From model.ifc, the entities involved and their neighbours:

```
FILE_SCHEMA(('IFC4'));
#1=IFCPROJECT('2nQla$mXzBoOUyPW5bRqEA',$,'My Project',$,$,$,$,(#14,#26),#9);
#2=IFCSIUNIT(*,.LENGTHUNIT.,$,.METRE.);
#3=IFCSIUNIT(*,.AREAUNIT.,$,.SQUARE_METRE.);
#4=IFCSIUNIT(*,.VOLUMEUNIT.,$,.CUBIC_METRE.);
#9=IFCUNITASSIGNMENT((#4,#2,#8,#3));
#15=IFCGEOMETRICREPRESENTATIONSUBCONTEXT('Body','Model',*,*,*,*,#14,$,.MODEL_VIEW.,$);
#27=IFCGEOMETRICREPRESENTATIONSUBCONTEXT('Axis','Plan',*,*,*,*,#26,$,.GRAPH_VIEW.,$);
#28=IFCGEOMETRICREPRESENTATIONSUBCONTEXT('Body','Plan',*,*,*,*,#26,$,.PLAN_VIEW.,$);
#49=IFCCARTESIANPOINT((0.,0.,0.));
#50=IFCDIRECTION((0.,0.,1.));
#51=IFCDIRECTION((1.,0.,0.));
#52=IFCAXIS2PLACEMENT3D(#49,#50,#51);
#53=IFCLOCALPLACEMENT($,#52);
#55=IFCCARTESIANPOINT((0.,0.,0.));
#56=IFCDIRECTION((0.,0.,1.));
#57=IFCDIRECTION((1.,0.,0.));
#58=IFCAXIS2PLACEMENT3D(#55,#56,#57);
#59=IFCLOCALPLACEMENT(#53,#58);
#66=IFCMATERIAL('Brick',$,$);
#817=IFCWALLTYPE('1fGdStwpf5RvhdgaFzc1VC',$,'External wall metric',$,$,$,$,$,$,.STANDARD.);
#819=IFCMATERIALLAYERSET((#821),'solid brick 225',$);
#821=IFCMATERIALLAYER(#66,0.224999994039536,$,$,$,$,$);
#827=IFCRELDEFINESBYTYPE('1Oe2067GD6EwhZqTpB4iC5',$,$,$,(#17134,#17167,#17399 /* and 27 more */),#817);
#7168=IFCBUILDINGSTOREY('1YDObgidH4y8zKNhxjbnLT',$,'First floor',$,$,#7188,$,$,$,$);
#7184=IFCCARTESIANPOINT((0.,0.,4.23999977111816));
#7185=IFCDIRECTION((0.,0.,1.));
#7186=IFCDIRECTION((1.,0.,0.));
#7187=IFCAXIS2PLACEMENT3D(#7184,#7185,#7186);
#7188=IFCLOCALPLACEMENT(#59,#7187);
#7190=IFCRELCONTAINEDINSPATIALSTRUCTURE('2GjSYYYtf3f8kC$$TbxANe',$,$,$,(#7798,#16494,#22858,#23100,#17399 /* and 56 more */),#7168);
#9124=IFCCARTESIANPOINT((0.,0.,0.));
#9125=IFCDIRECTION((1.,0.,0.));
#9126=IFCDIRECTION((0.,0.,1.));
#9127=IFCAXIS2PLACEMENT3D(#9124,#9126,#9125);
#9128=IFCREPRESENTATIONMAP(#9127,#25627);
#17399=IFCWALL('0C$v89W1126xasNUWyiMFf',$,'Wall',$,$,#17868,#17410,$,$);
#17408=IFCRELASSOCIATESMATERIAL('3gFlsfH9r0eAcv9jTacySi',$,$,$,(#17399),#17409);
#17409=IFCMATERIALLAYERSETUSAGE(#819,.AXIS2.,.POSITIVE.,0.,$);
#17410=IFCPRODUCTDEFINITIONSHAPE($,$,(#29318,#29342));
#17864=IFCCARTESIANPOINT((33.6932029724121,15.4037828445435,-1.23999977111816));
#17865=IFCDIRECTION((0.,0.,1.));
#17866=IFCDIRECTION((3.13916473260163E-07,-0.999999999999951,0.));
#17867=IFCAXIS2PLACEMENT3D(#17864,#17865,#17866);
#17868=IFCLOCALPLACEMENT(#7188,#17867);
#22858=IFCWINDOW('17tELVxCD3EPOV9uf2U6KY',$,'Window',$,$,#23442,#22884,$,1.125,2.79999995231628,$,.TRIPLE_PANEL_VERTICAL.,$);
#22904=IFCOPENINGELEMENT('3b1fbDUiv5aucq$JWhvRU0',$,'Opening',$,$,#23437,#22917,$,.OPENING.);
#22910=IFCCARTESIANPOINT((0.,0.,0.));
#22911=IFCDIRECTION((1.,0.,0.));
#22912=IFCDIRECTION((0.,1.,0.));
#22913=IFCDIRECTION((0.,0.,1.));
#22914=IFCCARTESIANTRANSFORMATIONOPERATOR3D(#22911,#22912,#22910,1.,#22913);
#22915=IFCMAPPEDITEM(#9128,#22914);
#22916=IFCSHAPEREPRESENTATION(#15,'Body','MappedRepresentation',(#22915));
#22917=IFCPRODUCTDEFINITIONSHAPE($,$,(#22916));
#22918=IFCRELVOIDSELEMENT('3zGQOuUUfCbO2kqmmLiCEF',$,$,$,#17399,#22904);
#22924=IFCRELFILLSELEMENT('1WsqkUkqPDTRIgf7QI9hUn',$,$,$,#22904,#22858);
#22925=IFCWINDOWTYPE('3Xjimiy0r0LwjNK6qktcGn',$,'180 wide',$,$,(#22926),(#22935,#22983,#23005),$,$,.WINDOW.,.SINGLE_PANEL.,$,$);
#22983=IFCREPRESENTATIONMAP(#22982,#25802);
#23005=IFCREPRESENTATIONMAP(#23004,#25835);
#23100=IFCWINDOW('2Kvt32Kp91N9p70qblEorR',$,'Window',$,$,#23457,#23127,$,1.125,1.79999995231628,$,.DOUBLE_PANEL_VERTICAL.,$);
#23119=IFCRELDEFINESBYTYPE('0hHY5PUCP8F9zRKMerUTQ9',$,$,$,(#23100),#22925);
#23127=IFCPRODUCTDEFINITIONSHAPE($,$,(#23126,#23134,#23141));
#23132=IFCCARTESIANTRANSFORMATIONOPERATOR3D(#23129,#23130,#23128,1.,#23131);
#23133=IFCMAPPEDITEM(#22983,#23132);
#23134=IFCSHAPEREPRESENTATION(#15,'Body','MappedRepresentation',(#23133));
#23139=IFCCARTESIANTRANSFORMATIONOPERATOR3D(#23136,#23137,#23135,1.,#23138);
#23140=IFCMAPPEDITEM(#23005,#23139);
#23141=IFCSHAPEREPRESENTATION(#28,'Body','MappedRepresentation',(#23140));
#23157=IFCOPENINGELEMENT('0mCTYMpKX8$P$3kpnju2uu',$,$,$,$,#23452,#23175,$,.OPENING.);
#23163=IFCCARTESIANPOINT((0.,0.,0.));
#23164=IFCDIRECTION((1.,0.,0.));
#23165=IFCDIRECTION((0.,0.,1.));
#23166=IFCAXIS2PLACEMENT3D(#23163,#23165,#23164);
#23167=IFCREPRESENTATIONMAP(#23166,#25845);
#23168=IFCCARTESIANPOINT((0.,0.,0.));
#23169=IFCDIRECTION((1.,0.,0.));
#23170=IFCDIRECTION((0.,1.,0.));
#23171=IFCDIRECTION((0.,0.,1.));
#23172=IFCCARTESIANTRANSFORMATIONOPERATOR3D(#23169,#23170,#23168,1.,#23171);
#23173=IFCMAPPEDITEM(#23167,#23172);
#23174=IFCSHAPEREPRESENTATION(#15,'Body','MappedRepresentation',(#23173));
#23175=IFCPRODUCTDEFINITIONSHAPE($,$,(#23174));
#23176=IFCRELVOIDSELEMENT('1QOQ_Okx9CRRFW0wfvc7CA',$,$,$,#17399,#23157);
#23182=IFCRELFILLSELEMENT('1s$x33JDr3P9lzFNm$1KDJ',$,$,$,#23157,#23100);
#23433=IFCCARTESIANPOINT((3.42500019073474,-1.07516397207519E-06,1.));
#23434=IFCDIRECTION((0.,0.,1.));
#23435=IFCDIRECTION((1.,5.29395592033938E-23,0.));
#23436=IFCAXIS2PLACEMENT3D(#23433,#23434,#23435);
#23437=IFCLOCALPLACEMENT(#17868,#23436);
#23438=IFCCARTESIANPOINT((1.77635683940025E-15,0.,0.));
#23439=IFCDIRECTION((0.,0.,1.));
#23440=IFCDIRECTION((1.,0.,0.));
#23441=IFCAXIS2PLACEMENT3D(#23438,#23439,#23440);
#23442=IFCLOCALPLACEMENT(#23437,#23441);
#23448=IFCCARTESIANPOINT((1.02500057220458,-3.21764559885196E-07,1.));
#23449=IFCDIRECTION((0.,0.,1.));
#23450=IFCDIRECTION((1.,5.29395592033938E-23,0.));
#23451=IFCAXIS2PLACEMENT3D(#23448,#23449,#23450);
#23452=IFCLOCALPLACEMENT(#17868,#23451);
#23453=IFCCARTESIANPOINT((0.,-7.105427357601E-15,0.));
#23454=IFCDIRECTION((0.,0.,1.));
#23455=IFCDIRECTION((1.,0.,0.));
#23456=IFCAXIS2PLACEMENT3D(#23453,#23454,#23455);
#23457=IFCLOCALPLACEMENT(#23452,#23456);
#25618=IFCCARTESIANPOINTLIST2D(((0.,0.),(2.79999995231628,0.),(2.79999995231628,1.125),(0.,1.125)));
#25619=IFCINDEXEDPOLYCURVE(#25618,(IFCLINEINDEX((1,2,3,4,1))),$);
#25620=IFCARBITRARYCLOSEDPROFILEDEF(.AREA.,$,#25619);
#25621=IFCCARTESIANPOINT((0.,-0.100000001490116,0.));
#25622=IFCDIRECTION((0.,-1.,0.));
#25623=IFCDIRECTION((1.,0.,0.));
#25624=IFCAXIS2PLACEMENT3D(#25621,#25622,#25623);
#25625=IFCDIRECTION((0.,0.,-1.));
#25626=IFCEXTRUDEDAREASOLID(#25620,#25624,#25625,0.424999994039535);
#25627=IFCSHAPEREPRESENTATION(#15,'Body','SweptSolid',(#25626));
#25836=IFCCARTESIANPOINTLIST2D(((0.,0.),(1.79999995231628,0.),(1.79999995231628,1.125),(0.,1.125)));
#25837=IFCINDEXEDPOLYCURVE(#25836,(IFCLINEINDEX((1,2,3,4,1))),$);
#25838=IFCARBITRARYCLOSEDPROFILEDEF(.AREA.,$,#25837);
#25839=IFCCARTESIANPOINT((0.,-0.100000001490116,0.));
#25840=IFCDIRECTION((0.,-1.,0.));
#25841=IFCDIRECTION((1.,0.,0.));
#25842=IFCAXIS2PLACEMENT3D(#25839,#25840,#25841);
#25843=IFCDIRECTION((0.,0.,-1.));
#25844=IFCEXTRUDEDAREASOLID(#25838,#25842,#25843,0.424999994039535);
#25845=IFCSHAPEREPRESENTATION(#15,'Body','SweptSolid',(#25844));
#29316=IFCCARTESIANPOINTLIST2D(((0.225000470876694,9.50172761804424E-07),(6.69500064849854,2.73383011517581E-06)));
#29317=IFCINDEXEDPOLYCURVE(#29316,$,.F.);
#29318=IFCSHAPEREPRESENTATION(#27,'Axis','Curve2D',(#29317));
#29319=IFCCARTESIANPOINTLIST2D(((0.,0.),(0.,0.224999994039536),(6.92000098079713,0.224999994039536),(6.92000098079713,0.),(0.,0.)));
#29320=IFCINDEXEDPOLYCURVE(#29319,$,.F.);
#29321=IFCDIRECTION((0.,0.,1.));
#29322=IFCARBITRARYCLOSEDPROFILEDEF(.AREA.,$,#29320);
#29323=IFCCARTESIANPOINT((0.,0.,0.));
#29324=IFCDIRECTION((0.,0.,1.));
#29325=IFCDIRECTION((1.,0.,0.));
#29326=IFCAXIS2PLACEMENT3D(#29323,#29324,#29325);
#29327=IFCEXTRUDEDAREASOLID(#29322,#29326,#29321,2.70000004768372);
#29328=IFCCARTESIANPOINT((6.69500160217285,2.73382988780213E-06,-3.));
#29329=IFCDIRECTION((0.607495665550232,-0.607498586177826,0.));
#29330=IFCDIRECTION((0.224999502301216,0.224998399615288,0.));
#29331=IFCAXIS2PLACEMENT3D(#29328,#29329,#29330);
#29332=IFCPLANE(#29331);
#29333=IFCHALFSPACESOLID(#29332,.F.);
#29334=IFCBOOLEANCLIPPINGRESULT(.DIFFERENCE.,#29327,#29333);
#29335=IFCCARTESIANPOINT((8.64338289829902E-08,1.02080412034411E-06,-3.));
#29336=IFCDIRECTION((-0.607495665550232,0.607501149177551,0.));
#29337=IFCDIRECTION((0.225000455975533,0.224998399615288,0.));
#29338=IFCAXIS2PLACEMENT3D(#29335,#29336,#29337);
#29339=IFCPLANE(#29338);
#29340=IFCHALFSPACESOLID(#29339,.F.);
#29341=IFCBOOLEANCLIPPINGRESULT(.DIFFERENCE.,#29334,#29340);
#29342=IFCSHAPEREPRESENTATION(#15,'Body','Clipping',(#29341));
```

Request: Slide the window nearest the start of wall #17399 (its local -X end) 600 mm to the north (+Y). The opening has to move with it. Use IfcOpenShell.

```python
import ifcopenshell
import ifcopenshell.api.geometry
import ifcopenshell.util.placement
import ifcopenshell.util.unit

model = ifcopenshell.open("model.ifc")
unit_scale = ifcopenshell.util.unit.calculate_unit_scale(model)

window = model.by_guid("2Kvt32Kp91N9p70qblEorR")
opening = window.FillsVoids[0].RelatingOpeningElement
wall = opening.VoidsElements[0].RelatingBuildingElement

wall_matrix = ifcopenshell.util.placement.get_local_placement(wall.ObjectPlacement)
shift = wall_matrix[:3, 0] * -0.6 / unit_scale
before = ifcopenshell.util.placement.get_local_placement(window.ObjectPlacement)[:3, 3].copy()

# The window is placed relative to its opening, so it follows when the opening moves.
matrix = ifcopenshell.util.placement.get_local_placement(opening.ObjectPlacement)
matrix[:3, 3] += shift
ifcopenshell.api.geometry.edit_object_placement(
    model, product=opening, matrix=matrix, is_si=False, should_transform_children=True
)

after = ifcopenshell.util.placement.get_local_placement(window.ObjectPlacement)[:3, 3]
print("window moved by", (after - before).round(3) + 0.0)

model.write("model_updated.ifc")
```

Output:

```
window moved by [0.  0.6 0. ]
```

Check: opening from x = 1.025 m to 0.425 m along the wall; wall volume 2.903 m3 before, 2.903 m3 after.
